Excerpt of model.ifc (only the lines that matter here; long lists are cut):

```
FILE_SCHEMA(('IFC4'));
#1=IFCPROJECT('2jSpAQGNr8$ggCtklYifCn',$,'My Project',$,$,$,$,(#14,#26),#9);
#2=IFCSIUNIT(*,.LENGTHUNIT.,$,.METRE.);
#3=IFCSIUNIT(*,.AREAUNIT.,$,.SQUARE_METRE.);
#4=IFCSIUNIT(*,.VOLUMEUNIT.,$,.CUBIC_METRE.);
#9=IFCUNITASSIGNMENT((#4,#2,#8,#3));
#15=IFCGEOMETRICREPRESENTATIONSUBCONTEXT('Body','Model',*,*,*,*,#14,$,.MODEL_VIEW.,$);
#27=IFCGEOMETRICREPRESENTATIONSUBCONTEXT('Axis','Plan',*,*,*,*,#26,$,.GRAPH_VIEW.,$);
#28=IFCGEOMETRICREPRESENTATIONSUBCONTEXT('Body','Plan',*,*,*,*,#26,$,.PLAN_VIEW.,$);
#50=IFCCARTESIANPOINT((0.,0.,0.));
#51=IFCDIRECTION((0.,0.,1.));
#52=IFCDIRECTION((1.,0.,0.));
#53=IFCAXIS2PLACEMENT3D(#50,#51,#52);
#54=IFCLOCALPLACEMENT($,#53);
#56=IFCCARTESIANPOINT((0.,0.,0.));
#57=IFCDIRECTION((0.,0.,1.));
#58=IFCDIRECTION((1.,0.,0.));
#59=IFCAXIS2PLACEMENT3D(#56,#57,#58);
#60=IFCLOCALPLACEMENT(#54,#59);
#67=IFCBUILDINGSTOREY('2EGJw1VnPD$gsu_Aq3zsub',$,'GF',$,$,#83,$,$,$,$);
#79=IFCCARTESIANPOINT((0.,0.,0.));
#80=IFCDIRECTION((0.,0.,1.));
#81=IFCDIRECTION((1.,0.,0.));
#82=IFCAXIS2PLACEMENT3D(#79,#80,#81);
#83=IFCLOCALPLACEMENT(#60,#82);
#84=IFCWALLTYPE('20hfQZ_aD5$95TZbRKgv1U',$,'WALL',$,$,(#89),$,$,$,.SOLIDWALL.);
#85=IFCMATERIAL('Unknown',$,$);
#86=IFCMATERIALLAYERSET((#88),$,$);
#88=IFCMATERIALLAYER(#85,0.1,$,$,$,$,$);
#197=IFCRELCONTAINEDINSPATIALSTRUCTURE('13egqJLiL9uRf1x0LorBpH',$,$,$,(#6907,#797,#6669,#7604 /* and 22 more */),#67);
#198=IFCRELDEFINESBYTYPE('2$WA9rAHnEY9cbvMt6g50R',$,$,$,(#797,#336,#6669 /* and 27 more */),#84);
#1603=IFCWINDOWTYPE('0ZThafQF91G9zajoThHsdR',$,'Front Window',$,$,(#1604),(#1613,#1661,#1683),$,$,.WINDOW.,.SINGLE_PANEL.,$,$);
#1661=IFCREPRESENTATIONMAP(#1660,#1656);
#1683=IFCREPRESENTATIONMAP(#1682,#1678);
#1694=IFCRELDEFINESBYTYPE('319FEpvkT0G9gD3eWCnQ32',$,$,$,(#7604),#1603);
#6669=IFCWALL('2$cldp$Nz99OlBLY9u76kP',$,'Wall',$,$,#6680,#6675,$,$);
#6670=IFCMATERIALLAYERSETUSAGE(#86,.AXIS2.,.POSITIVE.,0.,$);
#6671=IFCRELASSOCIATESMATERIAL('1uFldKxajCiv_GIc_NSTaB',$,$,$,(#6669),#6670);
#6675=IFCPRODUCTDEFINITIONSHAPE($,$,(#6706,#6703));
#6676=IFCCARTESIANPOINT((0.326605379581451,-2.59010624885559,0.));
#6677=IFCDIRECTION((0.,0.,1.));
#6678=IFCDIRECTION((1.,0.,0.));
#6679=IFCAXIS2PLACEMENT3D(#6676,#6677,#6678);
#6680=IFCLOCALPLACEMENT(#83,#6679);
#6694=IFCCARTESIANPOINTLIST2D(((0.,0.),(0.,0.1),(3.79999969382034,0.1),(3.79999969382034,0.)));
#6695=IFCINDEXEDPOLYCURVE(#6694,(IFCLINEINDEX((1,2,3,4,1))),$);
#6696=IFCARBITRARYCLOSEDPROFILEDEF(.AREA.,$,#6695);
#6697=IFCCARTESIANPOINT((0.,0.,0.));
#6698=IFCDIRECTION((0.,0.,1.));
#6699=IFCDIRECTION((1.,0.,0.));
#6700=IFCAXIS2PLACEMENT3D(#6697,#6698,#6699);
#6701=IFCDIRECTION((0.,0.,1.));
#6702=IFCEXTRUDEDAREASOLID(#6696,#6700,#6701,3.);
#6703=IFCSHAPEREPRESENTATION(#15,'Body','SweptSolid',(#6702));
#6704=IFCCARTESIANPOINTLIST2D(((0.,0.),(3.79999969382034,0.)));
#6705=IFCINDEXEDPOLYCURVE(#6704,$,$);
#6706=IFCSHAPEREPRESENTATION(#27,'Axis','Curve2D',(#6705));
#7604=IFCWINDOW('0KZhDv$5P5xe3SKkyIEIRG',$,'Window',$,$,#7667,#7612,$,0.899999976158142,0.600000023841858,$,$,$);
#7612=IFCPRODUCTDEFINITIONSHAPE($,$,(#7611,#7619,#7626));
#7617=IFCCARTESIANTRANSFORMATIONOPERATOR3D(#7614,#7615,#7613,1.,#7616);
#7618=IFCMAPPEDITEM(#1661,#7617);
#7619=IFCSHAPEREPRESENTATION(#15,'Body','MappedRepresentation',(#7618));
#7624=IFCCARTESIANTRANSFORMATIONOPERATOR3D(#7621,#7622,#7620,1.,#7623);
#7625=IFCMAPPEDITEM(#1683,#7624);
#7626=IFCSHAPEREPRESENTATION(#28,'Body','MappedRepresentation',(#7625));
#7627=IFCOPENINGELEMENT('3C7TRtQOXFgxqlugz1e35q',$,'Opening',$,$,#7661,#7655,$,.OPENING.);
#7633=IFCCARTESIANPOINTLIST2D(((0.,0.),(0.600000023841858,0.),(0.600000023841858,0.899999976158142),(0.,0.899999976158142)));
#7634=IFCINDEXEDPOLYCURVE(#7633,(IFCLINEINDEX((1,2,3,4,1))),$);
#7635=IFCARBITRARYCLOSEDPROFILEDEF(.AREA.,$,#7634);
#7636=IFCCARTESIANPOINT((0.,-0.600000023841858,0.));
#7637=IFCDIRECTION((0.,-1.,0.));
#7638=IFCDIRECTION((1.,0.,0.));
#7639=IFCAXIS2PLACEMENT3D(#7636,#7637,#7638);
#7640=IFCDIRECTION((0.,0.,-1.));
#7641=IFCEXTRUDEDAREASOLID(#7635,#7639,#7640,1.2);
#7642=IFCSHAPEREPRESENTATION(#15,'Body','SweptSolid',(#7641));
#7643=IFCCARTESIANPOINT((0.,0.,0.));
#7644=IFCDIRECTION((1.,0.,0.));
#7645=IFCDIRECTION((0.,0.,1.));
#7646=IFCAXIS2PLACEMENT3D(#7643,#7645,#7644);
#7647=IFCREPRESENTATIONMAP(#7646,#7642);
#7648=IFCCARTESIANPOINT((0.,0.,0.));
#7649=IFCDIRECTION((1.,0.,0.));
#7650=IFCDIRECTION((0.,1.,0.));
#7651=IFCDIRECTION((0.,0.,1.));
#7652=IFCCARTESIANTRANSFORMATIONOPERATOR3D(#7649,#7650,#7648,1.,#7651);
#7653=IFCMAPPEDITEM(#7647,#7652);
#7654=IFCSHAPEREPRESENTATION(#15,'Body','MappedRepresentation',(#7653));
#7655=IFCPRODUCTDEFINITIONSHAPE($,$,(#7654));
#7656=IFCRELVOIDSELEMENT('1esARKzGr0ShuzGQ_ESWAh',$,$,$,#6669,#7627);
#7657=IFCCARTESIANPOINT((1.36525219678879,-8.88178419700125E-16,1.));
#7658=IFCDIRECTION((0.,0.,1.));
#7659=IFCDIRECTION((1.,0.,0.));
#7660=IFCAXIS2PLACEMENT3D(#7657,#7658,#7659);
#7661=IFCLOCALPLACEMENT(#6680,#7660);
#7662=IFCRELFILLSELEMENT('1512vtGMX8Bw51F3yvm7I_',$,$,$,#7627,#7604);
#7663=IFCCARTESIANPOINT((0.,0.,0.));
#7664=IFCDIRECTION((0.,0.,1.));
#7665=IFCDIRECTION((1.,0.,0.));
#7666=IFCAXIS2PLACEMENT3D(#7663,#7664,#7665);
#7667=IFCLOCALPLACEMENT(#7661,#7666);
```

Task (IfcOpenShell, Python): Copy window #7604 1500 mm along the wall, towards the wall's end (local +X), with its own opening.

```python
import ifcopenshell
import ifcopenshell.api.feature
import ifcopenshell.api.geometry
import ifcopenshell.api.root
import ifcopenshell.geom
import ifcopenshell.util.element
import ifcopenshell.util.placement
import ifcopenshell.util.shape

model = ifcopenshell.open("model.ifc")
settings = ifcopenshell.geom.settings()


def volume(element):
    """Net volume in cubic metres, openings subtracted."""
    shape = ifcopenshell.geom.create_shape(settings, element)
    return ifcopenshell.util.shape.get_volume(shape.geometry)


window = model.by_id(7604)
opening = window.FillsVoids[0].RelatingOpeningElement
wall = opening.VoidsElements[0].RelatingBuildingElement
before = volume(wall)
shift = ifcopenshell.util.placement.get_local_placement(wall.ObjectPlacement)[:3, 0] * 1.5

# copy_class copies the void relationship, type, container and properties, but no geometry.
new_opening = ifcopenshell.api.root.copy_class(model, product=opening)
new_opening.Representation = ifcopenshell.util.element.copy_deep(
    model, opening.Representation, exclude=["IfcGeometricRepresentationContext", "IfcRepresentationMap"]
)
new_window = ifcopenshell.api.root.copy_class(model, product=window)
new_window.Representation = ifcopenshell.util.element.copy_deep(
    model, window.Representation, exclude=["IfcGeometricRepresentationContext", "IfcRepresentationMap"]
)
ifcopenshell.api.feature.add_filling(model, opening=new_opening, element=new_window)

for old, new in ((opening, new_opening), (window, new_window)):
    matrix = ifcopenshell.util.placement.get_local_placement(old.ObjectPlacement)
    matrix[:3, 3] += shift
    ifcopenshell.api.geometry.edit_object_placement(model, product=new, matrix=matrix, is_si=False)

after = volume(wall)

print(f"wall volume {before:.3f} -> {after:.3f} m3")

model.write("model_updated.ifc")
```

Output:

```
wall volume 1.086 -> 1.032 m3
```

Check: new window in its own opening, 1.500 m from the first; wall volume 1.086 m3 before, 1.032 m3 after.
